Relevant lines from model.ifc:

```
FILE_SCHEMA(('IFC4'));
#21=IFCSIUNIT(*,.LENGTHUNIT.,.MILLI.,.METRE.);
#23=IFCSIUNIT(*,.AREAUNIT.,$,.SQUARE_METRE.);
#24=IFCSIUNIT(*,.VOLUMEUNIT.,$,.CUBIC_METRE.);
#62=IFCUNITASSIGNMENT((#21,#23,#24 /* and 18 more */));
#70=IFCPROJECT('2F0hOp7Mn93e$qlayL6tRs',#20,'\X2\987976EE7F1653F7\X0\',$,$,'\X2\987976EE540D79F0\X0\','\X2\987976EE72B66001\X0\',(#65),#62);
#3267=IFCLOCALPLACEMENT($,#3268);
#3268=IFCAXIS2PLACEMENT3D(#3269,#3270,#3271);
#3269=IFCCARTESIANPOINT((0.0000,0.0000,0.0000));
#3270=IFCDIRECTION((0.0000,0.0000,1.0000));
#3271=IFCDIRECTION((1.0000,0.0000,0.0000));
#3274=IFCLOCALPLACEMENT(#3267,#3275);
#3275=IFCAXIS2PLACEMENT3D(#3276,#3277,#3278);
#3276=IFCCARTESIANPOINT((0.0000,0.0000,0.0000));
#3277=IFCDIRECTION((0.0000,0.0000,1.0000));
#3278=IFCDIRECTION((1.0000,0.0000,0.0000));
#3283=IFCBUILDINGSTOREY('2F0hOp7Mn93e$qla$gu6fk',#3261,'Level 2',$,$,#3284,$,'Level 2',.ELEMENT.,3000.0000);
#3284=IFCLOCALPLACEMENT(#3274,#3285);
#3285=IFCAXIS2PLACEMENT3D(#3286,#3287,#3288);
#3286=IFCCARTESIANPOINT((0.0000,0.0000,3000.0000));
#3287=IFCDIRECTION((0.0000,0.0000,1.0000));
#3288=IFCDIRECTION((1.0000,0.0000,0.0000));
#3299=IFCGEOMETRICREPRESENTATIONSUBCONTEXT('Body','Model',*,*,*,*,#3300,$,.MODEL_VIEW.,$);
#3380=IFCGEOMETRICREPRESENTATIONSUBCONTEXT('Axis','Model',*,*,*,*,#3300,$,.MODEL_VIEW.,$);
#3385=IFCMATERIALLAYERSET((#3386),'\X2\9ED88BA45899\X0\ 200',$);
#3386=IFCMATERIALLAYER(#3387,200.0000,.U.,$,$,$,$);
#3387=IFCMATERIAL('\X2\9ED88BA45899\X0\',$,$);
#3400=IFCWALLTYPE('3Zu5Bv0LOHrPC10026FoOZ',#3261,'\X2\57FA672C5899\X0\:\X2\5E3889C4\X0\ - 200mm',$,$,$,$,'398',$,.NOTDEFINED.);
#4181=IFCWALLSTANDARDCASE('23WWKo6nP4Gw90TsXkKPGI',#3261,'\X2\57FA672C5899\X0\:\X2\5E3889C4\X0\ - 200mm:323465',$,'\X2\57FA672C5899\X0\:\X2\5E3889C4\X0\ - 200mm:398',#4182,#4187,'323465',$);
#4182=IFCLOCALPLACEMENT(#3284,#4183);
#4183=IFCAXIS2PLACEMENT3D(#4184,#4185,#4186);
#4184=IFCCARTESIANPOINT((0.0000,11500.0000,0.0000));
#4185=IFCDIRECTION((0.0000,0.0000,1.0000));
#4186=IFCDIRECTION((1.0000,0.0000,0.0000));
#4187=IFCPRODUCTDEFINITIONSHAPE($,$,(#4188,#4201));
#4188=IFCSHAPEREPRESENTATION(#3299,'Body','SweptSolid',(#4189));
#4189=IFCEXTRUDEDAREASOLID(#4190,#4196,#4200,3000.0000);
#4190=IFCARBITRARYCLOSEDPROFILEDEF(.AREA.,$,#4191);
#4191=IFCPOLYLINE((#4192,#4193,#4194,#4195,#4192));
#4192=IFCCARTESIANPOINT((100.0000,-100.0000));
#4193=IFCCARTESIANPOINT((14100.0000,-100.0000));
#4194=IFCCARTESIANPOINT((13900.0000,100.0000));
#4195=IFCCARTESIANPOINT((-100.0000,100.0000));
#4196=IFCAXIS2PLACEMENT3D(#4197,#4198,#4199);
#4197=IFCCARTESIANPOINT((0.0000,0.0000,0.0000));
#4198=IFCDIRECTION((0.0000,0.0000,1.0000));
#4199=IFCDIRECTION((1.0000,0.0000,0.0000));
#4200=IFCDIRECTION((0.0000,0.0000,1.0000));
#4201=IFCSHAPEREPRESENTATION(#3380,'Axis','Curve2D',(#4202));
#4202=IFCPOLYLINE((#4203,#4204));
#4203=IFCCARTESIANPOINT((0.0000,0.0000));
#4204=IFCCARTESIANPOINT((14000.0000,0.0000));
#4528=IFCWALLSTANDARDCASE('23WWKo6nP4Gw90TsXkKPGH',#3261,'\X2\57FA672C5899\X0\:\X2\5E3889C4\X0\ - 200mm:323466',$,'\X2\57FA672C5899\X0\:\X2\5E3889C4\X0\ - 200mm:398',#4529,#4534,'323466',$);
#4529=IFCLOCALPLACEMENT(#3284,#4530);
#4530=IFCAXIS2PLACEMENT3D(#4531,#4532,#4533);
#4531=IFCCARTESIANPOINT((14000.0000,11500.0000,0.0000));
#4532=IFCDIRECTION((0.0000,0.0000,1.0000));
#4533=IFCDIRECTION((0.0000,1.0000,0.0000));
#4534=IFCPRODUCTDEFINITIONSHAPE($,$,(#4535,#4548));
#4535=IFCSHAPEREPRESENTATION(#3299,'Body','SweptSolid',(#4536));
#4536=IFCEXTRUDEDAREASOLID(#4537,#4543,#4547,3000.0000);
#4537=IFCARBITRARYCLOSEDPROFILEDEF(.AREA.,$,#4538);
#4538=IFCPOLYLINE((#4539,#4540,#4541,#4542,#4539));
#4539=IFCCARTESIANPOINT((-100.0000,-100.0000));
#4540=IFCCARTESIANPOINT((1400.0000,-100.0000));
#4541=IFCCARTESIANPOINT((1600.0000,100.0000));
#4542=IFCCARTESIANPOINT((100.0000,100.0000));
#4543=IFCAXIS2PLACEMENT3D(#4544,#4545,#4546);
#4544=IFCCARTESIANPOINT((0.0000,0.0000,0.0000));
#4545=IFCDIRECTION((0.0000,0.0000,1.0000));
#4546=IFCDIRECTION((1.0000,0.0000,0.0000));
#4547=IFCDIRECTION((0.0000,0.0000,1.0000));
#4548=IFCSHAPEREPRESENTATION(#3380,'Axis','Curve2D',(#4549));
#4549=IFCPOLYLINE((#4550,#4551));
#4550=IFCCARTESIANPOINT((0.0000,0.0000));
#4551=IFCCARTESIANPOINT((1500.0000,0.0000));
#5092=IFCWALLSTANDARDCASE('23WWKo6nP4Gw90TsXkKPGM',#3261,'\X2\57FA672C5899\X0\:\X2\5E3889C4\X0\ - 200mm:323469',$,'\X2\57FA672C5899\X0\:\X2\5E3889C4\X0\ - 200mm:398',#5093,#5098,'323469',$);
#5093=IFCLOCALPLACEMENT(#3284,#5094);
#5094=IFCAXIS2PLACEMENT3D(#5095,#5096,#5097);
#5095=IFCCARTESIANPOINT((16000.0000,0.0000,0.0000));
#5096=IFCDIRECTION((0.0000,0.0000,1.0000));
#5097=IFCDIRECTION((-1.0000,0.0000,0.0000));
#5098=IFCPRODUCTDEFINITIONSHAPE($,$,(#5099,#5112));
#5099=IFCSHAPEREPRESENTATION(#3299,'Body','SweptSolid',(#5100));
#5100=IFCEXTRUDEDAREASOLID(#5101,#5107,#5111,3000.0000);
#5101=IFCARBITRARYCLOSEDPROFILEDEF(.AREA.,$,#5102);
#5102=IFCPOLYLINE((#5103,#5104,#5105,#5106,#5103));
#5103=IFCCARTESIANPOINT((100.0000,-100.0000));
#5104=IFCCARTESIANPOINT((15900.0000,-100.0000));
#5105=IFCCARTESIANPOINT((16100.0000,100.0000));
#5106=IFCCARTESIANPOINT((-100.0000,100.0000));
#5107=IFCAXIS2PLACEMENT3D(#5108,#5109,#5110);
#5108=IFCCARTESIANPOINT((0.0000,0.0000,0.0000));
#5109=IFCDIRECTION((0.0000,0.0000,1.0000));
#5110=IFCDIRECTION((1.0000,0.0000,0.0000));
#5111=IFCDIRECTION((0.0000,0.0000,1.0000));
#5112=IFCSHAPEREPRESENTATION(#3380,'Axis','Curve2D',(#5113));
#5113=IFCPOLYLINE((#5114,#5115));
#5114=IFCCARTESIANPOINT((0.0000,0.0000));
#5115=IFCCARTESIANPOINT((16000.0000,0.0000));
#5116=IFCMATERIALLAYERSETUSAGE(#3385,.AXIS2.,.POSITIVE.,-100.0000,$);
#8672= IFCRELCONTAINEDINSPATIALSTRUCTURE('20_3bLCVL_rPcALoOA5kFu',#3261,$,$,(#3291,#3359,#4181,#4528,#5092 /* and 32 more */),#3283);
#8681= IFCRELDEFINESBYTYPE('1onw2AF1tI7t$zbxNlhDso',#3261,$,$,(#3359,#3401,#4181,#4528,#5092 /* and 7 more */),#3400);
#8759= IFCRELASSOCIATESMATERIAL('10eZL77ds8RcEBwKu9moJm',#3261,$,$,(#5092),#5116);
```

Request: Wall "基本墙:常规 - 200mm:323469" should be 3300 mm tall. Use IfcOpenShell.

```python
import ifcopenshell
import ifcopenshell.geom
import ifcopenshell.util.representation
import ifcopenshell.util.shape
import ifcopenshell.util.unit

model = ifcopenshell.open("model.ifc")
unit_scale = ifcopenshell.util.unit.calculate_unit_scale(model)
settings = ifcopenshell.geom.settings()


def volume(element):
    """Net volume in cubic metres, openings subtracted."""
    shape = ifcopenshell.geom.create_shape(settings, element)
    return ifcopenshell.util.shape.get_volume(shape.geometry)


wall = model.by_guid("23WWKo6nP4Gw90TsXkKPGM")
before = volume(wall)

body = ifcopenshell.util.representation.get_representation(wall, "Model", "Body")
solid = body.Items[0]
old_height = solid.Depth
solid.Depth = 3.3 / unit_scale
after = volume(wall)

print(f"height {old_height:g} -> {solid.Depth:g}, volume {before:.3f} -> {after:.3f} m3")

model.write("model-out.ifc")
```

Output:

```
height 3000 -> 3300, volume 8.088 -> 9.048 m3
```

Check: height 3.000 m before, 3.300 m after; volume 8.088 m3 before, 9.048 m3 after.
